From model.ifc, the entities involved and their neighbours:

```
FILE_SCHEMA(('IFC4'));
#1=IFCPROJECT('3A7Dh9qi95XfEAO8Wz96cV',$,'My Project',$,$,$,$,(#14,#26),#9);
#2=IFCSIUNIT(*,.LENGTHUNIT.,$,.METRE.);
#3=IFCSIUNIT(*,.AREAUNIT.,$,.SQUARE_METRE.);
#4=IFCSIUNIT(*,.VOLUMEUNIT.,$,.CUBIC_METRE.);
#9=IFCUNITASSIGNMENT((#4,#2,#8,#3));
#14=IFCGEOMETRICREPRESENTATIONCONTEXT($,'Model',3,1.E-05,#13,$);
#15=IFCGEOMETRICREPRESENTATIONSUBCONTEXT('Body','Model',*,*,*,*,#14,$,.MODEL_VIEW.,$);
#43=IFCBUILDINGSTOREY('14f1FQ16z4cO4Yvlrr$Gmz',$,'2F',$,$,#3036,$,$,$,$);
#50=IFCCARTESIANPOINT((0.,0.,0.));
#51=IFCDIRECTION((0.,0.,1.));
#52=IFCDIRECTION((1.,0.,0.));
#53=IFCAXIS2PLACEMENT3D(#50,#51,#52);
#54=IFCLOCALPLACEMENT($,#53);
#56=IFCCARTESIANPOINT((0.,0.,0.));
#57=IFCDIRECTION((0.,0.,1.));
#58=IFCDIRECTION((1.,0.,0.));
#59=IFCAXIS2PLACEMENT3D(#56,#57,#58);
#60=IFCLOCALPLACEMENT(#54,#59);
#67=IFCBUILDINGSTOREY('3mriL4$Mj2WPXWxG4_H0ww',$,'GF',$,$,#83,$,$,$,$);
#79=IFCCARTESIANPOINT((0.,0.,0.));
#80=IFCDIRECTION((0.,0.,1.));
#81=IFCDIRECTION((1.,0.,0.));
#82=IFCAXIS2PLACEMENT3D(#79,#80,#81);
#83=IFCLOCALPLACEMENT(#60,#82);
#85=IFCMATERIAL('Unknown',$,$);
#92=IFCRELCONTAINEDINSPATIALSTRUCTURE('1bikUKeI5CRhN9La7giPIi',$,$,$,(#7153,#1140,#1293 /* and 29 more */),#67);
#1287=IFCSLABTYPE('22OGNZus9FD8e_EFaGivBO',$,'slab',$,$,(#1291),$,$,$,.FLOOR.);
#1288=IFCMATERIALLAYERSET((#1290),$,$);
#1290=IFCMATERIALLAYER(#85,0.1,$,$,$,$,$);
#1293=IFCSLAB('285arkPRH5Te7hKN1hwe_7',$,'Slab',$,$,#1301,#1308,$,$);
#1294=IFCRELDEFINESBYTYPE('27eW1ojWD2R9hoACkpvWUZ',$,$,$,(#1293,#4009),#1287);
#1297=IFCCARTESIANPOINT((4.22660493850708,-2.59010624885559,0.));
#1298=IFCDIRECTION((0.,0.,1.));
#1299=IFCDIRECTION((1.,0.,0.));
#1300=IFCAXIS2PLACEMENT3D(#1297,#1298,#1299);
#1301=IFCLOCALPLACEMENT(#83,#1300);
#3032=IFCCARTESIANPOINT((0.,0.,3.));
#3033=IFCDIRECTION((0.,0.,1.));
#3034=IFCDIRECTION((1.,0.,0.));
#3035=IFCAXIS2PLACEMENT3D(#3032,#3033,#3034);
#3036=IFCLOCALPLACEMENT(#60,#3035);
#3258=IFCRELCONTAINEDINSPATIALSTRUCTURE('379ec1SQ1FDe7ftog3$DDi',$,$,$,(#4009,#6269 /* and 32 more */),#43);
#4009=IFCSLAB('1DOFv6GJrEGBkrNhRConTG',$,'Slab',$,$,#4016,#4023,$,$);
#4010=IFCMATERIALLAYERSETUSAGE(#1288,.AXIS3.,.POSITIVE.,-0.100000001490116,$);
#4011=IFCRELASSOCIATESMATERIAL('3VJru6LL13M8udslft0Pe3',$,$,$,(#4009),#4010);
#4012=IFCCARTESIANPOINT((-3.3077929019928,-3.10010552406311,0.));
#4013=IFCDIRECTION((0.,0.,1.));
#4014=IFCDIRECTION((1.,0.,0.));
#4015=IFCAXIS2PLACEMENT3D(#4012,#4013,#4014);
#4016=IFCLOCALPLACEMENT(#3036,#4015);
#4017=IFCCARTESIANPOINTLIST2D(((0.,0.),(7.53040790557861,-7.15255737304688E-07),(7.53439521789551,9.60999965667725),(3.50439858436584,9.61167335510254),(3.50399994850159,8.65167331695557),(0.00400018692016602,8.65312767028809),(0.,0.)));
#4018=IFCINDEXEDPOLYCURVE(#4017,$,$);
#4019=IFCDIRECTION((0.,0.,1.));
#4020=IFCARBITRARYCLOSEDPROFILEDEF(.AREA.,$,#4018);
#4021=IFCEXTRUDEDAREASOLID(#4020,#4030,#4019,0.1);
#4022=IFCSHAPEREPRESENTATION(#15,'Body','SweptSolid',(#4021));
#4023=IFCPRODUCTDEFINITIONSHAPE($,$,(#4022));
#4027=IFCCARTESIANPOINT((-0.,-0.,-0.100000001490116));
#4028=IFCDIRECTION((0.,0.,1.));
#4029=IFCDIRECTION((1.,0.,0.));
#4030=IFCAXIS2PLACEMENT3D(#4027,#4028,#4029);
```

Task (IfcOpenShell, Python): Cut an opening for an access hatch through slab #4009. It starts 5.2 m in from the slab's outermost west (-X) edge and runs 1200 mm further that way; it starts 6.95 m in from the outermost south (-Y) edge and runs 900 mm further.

```python
import numpy as np
import ifcopenshell
import ifcopenshell.api.feature
import ifcopenshell.api.geometry
import ifcopenshell.api.root
import ifcopenshell.geom
import ifcopenshell.util.placement
import ifcopenshell.util.representation
import ifcopenshell.util.shape
import ifcopenshell.util.unit

model = ifcopenshell.open("model.ifc")
unit_scale = ifcopenshell.util.unit.calculate_unit_scale(model)
settings = ifcopenshell.geom.settings()


def volume(element):
    """Net volume in cubic metres, openings subtracted."""
    shape = ifcopenshell.geom.create_shape(settings, element)
    return ifcopenshell.util.shape.get_volume(shape.geometry)


slab = model.by_id(4009)
before = volume(slab)

# Extent in the slab's own axes, in metres. The edges named are its -X and -Y sides.
slab_shape = ifcopenshell.geom.create_shape(settings, slab)
vertices = ifcopenshell.util.shape.get_vertices(slab_shape.geometry)
x_min, y_min, bottom = vertices.min(axis=0)
top = vertices[:, 2].max()

opening = ifcopenshell.api.root.create_entity(model, ifc_class="IfcOpeningElement", name="Access hatch opening", predefined_type="OPENING")
context = ifcopenshell.util.representation.get_context(model, "Model", "Body", "MODEL_VIEW")
width, depth = 1.2, 0.9
outline = [(0.0, 0.0), (width, 0.0), (width, depth), (0.0, depth), (0.0, 0.0)]
# Overshoot both faces by 50 mm so the cut is clean.
shape = ifcopenshell.api.geometry.add_slab_representation(
    model, context=context, depth=top - bottom + 0.1, polyline=outline
)
ifcopenshell.api.geometry.assign_representation(model, product=opening, representation=shape)

matrix = ifcopenshell.util.placement.get_local_placement(slab.ObjectPlacement)
matrix[:, 3] = matrix @ np.append(np.array([x_min + 5.2, y_min + 6.95, bottom - 0.05]) / unit_scale, 1.0)
ifcopenshell.api.geometry.edit_object_placement(model, product=opening, matrix=matrix, is_si=False)
ifcopenshell.api.feature.add_feature(model, feature=opening, element=slab)

after = volume(slab)

print(f"slab volume {before:.3f} -> {after:.3f} m3")

model.write("model-out.ifc")
```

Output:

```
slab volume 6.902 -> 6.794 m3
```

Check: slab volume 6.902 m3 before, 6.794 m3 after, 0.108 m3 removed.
